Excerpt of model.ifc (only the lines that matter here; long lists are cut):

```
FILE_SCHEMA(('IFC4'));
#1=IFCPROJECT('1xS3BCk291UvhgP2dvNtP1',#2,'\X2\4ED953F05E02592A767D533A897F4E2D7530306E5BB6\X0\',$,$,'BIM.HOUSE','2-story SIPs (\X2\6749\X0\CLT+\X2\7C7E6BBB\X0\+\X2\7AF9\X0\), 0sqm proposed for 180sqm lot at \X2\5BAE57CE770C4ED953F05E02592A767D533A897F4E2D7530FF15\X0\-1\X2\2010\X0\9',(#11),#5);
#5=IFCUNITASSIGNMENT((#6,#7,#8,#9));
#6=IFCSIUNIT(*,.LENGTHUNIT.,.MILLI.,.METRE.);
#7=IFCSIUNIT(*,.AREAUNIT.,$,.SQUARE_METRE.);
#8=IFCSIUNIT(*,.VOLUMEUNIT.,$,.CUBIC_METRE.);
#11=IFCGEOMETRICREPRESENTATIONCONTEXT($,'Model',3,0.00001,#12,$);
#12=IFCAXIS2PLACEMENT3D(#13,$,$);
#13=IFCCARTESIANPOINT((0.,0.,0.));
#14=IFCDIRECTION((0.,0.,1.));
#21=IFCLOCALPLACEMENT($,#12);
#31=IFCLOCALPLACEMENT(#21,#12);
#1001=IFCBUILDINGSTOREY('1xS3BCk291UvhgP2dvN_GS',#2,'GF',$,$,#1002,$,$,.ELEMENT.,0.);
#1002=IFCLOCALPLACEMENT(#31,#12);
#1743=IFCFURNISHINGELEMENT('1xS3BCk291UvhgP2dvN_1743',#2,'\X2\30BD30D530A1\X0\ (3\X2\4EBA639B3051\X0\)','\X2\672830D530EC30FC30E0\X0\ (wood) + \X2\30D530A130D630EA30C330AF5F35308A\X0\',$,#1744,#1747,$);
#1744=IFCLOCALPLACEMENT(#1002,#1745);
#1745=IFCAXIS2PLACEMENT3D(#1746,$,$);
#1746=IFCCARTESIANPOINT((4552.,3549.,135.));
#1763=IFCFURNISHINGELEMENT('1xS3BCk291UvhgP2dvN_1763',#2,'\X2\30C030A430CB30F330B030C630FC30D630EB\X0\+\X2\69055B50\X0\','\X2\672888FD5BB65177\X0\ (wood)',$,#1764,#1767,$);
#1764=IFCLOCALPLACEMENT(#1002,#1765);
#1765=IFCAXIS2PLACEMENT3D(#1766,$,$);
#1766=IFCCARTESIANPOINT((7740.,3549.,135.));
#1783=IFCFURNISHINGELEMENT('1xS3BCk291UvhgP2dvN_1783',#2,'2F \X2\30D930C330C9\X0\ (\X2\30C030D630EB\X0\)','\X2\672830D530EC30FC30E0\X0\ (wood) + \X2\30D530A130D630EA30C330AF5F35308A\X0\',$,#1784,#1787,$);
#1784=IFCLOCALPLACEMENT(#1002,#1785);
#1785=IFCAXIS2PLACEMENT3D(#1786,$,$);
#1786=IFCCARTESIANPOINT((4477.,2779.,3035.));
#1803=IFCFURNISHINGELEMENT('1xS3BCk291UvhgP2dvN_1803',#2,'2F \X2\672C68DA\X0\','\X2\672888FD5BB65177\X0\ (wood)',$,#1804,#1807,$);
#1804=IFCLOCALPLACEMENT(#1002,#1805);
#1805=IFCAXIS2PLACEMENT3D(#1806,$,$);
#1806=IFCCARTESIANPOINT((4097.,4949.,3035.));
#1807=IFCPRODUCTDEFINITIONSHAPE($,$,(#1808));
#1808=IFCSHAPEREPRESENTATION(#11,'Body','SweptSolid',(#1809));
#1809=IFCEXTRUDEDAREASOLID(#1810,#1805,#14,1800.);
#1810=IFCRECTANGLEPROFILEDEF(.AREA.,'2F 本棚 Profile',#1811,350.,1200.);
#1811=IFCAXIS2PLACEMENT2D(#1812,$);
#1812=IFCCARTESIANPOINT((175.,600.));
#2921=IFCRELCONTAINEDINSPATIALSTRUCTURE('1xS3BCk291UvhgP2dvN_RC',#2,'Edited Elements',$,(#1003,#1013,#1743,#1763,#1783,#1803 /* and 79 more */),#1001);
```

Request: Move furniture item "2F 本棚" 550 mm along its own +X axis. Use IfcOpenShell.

```python
import ifcopenshell
import ifcopenshell.api.geometry
import ifcopenshell.util.placement
import ifcopenshell.util.unit

model = ifcopenshell.open("model.ifc")
unit_scale = ifcopenshell.util.unit.calculate_unit_scale(model)

item = model.by_guid("1xS3BCk291UvhgP2dvN_1803")
matrix = ifcopenshell.util.placement.get_local_placement(item.ObjectPlacement)
matrix[:3, 3] += matrix[:3, 0] * 0.55 / unit_scale
ifcopenshell.api.geometry.edit_object_placement(model, product=item, matrix=matrix, is_si=False)

print(ifcopenshell.util.placement.get_local_placement(item.ObjectPlacement).round(3) + 0.0)

model.write("model_v2.ifc")
```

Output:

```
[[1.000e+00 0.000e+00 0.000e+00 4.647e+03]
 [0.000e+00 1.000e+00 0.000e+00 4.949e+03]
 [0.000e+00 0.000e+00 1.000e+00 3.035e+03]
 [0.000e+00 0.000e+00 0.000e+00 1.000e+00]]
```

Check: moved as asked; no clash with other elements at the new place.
